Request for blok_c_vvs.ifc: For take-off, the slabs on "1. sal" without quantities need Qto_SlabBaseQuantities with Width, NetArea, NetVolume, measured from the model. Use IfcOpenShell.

First a look at what the model holds.

```python
import ifcopenshell
import ifcopenshell.util.element
import ifcopenshell.util.unit

model = ifcopenshell.open("blok_c_vvs.ifc")
print(model.schema)
for unit_type in ("LENGTHUNIT", "AREAUNIT", "VOLUMEUNIT"):
    print(unit_type, ifcopenshell.util.unit.calculate_unit_scale(model, unit_type))
storey = next(s for s in model.by_type("IfcBuildingStorey") if s.Name == "1. sal")
slabs = [e for e in ifcopenshell.util.element.get_decomposition(storey) if e.is_a("IfcSlab")]
for e in sorted(slabs, key=lambda e: e.id()):
    print(e.id(), e.is_a(), e.Name, list(ifcopenshell.util.element.get_psets(e, qtos_only=True)), sep=" | ")
```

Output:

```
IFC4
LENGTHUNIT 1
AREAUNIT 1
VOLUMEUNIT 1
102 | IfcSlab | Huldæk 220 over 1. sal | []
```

```python
import ifcopenshell
import ifcopenshell.api.pset
import ifcopenshell.geom
import ifcopenshell.util.element
import ifcopenshell.util.shape
import ifcopenshell.util.unit

model = ifcopenshell.open("blok_c_vvs.ifc")
unit_scale = ifcopenshell.util.unit.calculate_unit_scale(model)
area_scale = ifcopenshell.util.unit.calculate_unit_scale(model, "AREAUNIT")
volume_scale = ifcopenshell.util.unit.calculate_unit_scale(model, "VOLUMEUNIT")
settings = ifcopenshell.geom.settings()

storey = next(s for s in model.by_type("IfcBuildingStorey") if s.Name == "1. sal")
slabs = [e for e in ifcopenshell.util.element.get_decomposition(storey) if e.is_a("IfcSlab")]

for e in sorted(slabs, key=lambda e: e.id()):
    if ifcopenshell.util.element.get_psets(e, qtos_only=True, should_inherit=False):
        continue
    # Geometry comes back in metres, in the element's own axes.
    shape = ifcopenshell.geom.create_shape(settings, e)
    values = {
        "Width": ifcopenshell.util.shape.get_z(shape.geometry) / unit_scale,
        "NetArea": ifcopenshell.util.shape.get_footprint_area(shape.geometry) / area_scale,
        "NetVolume": ifcopenshell.util.shape.get_volume(shape.geometry) / volume_scale,
    }
    qto = ifcopenshell.api.pset.add_qto(model, product=e, name="Qto_SlabBaseQuantities")
    ifcopenshell.api.pset.edit_qto(model, qto=qto, properties=values)
    print(e.id(), {k: round(v, 3) for k, v in values.items()})

model.write("blok_c_vvs-out.ifc")
```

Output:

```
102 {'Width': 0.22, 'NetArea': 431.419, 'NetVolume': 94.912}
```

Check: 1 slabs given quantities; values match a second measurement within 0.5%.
